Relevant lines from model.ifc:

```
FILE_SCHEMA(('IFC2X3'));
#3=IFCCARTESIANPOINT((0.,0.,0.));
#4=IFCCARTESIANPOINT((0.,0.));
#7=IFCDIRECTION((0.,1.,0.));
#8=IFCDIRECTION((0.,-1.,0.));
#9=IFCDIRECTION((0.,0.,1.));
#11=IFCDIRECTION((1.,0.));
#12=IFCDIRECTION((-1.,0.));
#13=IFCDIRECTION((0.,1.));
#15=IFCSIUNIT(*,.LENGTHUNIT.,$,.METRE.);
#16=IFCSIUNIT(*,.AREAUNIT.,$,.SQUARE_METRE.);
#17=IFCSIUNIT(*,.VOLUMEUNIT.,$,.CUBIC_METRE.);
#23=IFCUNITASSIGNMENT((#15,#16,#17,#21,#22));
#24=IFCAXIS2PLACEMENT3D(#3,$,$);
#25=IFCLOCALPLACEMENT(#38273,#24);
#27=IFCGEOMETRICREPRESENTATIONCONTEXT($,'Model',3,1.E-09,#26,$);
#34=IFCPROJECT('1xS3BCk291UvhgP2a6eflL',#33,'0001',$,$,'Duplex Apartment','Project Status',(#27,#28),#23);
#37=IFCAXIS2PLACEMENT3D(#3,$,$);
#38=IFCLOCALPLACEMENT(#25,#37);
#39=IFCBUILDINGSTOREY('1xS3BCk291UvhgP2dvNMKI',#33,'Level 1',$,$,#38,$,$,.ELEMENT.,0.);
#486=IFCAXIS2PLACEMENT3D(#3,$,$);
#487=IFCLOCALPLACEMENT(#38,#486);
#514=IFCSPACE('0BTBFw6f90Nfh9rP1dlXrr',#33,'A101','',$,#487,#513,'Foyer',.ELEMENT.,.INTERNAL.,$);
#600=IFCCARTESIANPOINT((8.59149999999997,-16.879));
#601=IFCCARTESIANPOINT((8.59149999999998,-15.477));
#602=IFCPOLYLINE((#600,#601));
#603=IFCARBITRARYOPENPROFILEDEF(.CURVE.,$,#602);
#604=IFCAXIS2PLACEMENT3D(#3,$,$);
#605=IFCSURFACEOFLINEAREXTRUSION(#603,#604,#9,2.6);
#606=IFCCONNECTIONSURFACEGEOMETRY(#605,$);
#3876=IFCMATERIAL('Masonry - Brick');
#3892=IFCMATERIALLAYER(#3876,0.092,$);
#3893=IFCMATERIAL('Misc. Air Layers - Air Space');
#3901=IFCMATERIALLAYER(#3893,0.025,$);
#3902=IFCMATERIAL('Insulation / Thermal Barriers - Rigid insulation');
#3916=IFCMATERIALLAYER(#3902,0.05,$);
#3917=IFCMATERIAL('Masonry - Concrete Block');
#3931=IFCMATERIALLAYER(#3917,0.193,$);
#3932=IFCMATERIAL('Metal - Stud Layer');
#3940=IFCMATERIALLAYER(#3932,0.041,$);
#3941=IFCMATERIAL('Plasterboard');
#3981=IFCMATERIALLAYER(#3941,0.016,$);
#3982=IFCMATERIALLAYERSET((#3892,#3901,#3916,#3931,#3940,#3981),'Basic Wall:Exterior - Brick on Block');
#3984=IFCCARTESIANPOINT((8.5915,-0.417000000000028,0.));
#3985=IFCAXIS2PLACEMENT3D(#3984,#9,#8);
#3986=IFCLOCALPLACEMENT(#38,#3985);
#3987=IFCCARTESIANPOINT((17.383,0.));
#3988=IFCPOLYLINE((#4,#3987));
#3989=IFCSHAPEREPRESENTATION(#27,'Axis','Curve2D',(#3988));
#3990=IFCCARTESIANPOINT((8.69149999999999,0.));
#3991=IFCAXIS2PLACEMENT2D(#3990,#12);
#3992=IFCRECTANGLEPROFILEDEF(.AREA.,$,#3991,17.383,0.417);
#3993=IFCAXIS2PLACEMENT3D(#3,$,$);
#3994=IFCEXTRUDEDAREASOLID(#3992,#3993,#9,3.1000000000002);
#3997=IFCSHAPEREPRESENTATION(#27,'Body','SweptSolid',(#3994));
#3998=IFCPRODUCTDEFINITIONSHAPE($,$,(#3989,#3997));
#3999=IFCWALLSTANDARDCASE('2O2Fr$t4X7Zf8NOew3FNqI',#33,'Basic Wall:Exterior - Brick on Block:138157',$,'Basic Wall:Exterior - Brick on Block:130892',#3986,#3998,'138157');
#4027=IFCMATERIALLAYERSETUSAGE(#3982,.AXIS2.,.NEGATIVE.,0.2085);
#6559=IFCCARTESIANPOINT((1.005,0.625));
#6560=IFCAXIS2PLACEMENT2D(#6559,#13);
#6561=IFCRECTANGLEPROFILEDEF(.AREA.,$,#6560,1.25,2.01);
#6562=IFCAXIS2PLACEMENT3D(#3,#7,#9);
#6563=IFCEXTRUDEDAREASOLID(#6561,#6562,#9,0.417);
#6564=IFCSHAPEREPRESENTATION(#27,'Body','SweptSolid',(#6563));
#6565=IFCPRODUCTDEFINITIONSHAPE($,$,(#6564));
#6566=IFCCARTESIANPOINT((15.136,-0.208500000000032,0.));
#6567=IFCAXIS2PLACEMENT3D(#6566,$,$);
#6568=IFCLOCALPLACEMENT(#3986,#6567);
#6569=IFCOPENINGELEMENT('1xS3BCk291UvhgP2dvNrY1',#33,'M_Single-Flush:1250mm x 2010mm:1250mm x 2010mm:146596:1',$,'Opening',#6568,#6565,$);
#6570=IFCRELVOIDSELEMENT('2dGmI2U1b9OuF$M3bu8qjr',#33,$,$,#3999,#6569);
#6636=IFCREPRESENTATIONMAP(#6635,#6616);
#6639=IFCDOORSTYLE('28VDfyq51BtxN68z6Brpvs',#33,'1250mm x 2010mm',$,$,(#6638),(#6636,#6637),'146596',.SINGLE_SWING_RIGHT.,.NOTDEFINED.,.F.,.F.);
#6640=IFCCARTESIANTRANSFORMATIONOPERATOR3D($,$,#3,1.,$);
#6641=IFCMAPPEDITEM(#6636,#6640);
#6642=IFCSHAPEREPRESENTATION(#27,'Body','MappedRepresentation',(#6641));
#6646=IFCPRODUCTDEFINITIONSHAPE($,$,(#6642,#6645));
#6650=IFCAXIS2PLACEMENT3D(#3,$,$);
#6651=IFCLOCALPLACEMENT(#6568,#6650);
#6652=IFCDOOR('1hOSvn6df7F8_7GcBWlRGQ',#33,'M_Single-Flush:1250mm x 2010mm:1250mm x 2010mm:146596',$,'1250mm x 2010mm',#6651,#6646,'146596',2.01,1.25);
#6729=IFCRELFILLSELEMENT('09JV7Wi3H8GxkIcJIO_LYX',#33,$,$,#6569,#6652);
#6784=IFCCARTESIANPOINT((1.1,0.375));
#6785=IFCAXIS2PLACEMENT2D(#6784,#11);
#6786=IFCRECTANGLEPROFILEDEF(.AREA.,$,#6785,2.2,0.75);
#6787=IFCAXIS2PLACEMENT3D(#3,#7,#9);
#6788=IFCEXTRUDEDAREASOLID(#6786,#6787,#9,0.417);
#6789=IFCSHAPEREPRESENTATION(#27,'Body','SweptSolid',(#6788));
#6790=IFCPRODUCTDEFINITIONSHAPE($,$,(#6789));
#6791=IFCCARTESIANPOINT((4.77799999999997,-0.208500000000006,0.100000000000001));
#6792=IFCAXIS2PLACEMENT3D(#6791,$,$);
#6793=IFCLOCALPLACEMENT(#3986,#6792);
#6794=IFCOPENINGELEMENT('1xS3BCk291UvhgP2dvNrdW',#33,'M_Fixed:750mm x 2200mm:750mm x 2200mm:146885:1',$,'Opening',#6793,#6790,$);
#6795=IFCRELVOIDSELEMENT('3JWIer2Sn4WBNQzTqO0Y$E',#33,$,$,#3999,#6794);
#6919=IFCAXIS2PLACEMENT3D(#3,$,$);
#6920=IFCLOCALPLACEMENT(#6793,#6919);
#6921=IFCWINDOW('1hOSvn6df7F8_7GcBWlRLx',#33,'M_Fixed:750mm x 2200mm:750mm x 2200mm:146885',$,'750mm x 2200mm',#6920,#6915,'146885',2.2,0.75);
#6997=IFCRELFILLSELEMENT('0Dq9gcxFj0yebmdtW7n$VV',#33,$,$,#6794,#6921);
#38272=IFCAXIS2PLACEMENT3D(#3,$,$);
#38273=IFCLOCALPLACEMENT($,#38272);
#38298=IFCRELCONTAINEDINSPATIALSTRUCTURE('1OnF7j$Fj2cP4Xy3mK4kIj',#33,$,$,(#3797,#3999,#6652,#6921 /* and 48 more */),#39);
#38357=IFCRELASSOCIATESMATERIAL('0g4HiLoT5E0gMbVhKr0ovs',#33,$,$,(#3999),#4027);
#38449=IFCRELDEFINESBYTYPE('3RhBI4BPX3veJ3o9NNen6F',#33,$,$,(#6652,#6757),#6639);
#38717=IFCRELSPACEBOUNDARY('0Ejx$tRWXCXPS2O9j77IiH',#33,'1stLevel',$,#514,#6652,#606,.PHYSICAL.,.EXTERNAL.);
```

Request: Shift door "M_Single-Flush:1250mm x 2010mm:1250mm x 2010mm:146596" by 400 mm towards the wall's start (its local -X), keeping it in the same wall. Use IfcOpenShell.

```python
import numpy as np
import ifcopenshell
import ifcopenshell.api.geometry
import ifcopenshell.util.placement
import ifcopenshell.util.unit

model = ifcopenshell.open("model.ifc")
unit_scale = ifcopenshell.util.unit.calculate_unit_scale(model)

door = model.by_guid("1hOSvn6df7F8_7GcBWlRGQ")
opening = door.FillsVoids[0].RelatingOpeningElement
wall = opening.VoidsElements[0].RelatingBuildingElement

wall_matrix = ifcopenshell.util.placement.get_local_placement(wall.ObjectPlacement)
shift = wall_matrix[:3, 0] * -0.4 / unit_scale
before = ifcopenshell.util.placement.get_local_placement(door.ObjectPlacement)[:3, 3].copy()

# The door is placed relative to its opening, so it follows when the opening moves.
matrix = ifcopenshell.util.placement.get_local_placement(opening.ObjectPlacement)
matrix[:3, 3] += shift
ifcopenshell.api.geometry.edit_object_placement(
    model, product=opening, matrix=matrix, is_si=False, should_transform_children=True
)

# Space boundary surfaces are stored in each space's coordinates; move them too.
for rel in door.ProvidesBoundaries:
    if not rel.ConnectionGeometry:
        continue
    surface = rel.ConnectionGeometry.SurfaceOnRelatingElement
    space_matrix = ifcopenshell.util.placement.get_local_placement(rel.RelatingSpace.ObjectPlacement)
    point = np.array(surface.Position.Location.Coordinates) + space_matrix[:3, :3].T @ shift
    surface.Position = model.createIfcAxis2Placement3D(
        model.createIfcCartesianPoint(point.tolist()), surface.Position.Axis, surface.Position.RefDirection
    )

after = ifcopenshell.util.placement.get_local_placement(door.ObjectPlacement)[:3, 3]
print("door moved by", (after - before).round(3) + 0.0)

model.write("model-out.ifc")
```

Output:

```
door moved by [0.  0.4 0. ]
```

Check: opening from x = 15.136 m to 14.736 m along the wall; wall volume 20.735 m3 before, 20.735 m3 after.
